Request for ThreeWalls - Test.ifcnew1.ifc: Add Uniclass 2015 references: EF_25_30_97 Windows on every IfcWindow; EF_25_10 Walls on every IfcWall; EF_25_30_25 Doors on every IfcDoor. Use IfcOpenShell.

First a look at what the model holds.

```python
import ifcopenshell

model = ifcopenshell.open("ThreeWalls - Test.ifcnew1.ifc")
print(model.schema)
print("classifications:", [c.Name for c in model.by_type("IfcClassification")])
for ifc_class in ("IfcDoor", "IfcRoof", "IfcStair", "IfcWall", "IfcWindow"):
    print(ifc_class, len(model.by_type(ifc_class)))
```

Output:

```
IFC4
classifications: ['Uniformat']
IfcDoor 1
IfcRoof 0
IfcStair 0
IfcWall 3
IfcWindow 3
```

```python
import ifcopenshell
import ifcopenshell.api.classification

model = ifcopenshell.open("ThreeWalls - Test.ifcnew1.ifc")

system = ifcopenshell.api.classification.add_classification(model, classification="Uniclass 2015")

codes = {
    "IfcWindow": ("EF_25_30_97", "Windows"),
    "IfcWall": ("EF_25_10", "Walls"),
    "IfcDoor": ("EF_25_30_25", "Doors"),
}
for ifc_class, (code, name) in codes.items():
    products = model.by_type(ifc_class)
    ifcopenshell.api.classification.add_reference(
        model, products=products, classification=system, identification=code, name=name
    )
    print(code, len(products))

model.write("ThreeWalls - Test.ifcnew1_updated.ifc")
```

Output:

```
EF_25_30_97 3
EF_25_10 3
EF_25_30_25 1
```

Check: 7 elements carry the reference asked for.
